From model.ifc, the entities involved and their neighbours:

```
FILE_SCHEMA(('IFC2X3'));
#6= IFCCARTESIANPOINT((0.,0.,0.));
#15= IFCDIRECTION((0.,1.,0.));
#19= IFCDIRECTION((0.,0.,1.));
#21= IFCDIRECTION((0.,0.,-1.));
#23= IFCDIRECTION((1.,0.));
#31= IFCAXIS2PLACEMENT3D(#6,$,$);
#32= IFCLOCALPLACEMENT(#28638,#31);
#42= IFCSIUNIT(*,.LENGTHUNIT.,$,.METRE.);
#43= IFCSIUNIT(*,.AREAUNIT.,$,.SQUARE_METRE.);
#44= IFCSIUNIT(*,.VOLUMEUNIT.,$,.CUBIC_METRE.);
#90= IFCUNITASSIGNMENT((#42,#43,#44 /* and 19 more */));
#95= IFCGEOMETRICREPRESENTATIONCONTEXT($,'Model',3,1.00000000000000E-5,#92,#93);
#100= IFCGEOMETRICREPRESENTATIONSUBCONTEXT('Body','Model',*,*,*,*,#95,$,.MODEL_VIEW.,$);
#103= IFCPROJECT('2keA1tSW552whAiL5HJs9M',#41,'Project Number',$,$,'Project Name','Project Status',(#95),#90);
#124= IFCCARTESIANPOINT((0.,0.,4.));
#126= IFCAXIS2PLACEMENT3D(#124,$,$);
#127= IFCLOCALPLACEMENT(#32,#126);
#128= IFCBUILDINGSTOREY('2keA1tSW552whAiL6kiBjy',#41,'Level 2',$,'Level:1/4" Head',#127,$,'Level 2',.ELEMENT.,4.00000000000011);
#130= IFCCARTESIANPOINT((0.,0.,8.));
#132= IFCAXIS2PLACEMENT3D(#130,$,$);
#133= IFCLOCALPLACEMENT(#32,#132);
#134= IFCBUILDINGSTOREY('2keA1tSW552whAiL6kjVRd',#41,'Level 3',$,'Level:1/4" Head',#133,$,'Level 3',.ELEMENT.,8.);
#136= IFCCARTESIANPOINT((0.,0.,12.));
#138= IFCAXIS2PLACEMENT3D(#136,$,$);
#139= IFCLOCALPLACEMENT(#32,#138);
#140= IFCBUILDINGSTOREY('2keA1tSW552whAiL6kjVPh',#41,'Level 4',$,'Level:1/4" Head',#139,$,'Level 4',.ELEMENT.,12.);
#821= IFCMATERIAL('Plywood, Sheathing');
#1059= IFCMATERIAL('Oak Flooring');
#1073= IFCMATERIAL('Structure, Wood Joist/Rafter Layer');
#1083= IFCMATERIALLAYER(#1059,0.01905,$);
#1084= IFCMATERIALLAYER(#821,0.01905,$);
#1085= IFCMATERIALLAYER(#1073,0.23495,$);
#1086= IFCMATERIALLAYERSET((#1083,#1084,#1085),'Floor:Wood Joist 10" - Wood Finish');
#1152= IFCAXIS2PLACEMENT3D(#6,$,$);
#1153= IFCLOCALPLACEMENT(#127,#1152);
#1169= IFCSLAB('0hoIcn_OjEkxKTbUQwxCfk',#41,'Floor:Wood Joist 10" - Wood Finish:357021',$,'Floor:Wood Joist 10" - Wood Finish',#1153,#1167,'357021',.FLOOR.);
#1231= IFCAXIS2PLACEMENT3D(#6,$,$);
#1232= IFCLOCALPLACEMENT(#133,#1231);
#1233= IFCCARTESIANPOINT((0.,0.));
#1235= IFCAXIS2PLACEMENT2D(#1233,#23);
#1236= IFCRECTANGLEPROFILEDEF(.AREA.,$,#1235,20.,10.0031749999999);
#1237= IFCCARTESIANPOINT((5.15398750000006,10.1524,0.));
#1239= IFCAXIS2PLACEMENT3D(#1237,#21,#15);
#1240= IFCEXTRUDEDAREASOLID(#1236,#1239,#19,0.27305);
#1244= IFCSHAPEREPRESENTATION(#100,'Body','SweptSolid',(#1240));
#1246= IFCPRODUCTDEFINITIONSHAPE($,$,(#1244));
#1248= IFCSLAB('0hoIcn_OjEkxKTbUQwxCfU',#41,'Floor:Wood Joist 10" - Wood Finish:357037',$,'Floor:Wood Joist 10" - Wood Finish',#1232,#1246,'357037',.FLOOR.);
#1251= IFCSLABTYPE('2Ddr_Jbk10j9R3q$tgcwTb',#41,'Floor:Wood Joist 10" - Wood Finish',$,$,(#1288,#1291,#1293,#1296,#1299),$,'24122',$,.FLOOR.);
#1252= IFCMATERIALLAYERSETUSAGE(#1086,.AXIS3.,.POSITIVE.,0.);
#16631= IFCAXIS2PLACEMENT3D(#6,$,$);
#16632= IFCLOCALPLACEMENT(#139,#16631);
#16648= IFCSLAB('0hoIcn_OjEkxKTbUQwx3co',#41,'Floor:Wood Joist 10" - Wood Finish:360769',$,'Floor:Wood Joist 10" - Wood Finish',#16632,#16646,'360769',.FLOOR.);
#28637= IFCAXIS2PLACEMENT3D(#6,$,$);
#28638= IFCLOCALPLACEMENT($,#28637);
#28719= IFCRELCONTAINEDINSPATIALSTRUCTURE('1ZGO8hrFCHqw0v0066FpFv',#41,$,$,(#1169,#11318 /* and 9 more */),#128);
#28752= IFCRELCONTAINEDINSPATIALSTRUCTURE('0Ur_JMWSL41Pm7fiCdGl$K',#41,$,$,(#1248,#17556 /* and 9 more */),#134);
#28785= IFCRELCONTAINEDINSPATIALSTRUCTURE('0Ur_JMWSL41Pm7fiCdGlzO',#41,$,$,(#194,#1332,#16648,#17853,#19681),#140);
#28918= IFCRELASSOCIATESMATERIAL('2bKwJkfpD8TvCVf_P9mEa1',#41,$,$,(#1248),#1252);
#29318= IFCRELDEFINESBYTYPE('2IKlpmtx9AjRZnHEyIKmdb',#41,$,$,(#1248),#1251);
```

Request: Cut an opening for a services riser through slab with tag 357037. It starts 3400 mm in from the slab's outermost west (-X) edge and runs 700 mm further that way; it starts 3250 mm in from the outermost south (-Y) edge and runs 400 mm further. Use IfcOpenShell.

```python
import numpy as np
import ifcopenshell
import ifcopenshell.api.feature
import ifcopenshell.api.geometry
import ifcopenshell.api.root
import ifcopenshell.geom
import ifcopenshell.util.placement
import ifcopenshell.util.representation
import ifcopenshell.util.shape
import ifcopenshell.util.unit

model = ifcopenshell.open("model.ifc")
unit_scale = ifcopenshell.util.unit.calculate_unit_scale(model)
settings = ifcopenshell.geom.settings()


def volume(element):
    """Net volume in cubic metres, openings subtracted."""
    shape = ifcopenshell.geom.create_shape(settings, element)
    return ifcopenshell.util.shape.get_volume(shape.geometry)


slab = model.by_id(1248)
before = volume(slab)

# Extent in the slab's own axes, in metres. The edges named are its -X and -Y sides.
slab_shape = ifcopenshell.geom.create_shape(settings, slab)
vertices = ifcopenshell.util.shape.get_vertices(slab_shape.geometry)
x_min, y_min, bottom = vertices.min(axis=0)
top = vertices[:, 2].max()

opening = ifcopenshell.api.root.create_entity(model, ifc_class="IfcOpeningElement", name="Services riser opening")
context = ifcopenshell.util.representation.get_context(model, "Model", "Body", "MODEL_VIEW")
width, depth = 0.7, 0.4
outline = [(0.0, 0.0), (width, 0.0), (width, depth), (0.0, depth), (0.0, 0.0)]
# Overshoot both faces by 50 mm so the cut is clean.
shape = ifcopenshell.api.geometry.add_slab_representation(
    model, context=context, depth=top - bottom + 0.1, polyline=outline
)
ifcopenshell.api.geometry.assign_representation(model, product=opening, representation=shape)

matrix = ifcopenshell.util.placement.get_local_placement(slab.ObjectPlacement)
matrix[:, 3] = matrix @ np.append(np.array([x_min + 3.4, y_min + 3.25, bottom - 0.05]) / unit_scale, 1.0)
ifcopenshell.api.geometry.edit_object_placement(model, product=opening, matrix=matrix, is_si=False)
ifcopenshell.api.feature.add_feature(model, feature=opening, element=slab)

after = volume(slab)

print(f"slab volume {before:.3f} -> {after:.3f} m3")

model.write("model-out.ifc")
```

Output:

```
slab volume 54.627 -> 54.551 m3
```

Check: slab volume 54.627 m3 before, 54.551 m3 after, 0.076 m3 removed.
